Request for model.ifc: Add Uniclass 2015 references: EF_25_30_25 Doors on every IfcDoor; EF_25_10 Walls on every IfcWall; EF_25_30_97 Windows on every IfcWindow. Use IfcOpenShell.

First a look at what the model holds.

```python
import ifcopenshell

model = ifcopenshell.open("model.ifc")
print(model.schema)
print("classifications:", [c.Name for c in model.by_type("IfcClassification")])
for ifc_class in ("IfcDoor", "IfcRoof", "IfcStair", "IfcWall", "IfcWindow"):
    print(ifc_class, len(model.by_type(ifc_class)))
```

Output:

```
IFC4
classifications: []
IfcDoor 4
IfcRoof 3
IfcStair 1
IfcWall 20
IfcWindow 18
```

```python
import ifcopenshell
import ifcopenshell.api.classification

model = ifcopenshell.open("model.ifc")

system = ifcopenshell.api.classification.add_classification(model, classification="Uniclass 2015")

codes = {
    "IfcDoor": ("EF_25_30_25", "Doors"),
    "IfcWall": ("EF_25_10", "Walls"),
    "IfcWindow": ("EF_25_30_97", "Windows"),
}
for ifc_class, (code, name) in codes.items():
    products = model.by_type(ifc_class)
    ifcopenshell.api.classification.add_reference(
        model, products=products, classification=system, identification=code, name=name
    )
    print(code, len(products))

model.write("model_rev.ifc")
```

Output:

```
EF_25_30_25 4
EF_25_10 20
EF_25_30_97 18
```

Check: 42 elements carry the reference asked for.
